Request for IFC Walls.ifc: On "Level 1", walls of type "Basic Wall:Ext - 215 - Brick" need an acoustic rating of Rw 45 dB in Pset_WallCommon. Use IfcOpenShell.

First a look at what the model holds.

```python
import ifcopenshell
import ifcopenshell.util.element

model = ifcopenshell.open("IFC Walls.ifc")
print(model.schema)
storey = next(s for s in model.by_type("IfcBuildingStorey") if s.Name == "Level 1")
walls = [e for e in ifcopenshell.util.element.get_decomposition(storey) if e.is_a("IfcWall")]
seen = {}
for e in walls:
    element_type = ifcopenshell.util.element.get_type(e)
    key = (element_type.Name if element_type != e and element_type else None, ifcopenshell.util.element.get_pset(e, "Pset_WallCommon", "AcousticRating"))
    seen[key] = seen.get(key, 0) + 1
for (name, value), count in sorted(seen.items(), key=str):
    print(count, "x", name, "|", value)
```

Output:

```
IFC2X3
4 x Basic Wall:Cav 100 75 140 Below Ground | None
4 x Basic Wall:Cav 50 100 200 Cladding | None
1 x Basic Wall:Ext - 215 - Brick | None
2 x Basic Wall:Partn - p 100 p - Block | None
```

```python
import ifcopenshell
import ifcopenshell.api.pset
import ifcopenshell.util.element

model = ifcopenshell.open("IFC Walls.ifc")

storey = next(s for s in model.by_type("IfcBuildingStorey") if s.Name == "Level 1")
walls = [e for e in ifcopenshell.util.element.get_decomposition(storey) if e.is_a("IfcWall")]

count = 0
for e in walls:
    element_type = ifcopenshell.util.element.get_type(e)
    if element_type in (None, e) or element_type.Name != "Basic Wall:Ext - 215 - Brick":
        continue
    # add_pset returns the element's existing set when there is one.
    pset = ifcopenshell.api.pset.add_pset(model, product=e, name="Pset_WallCommon")
    ifcopenshell.api.pset.edit_pset(model, pset=pset, properties={"AcousticRating": "Rw 45 dB"})
    count += 1

print(count, "walls updated")

model.write("IFC Walls_rev.ifc")
```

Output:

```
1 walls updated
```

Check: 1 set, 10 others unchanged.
